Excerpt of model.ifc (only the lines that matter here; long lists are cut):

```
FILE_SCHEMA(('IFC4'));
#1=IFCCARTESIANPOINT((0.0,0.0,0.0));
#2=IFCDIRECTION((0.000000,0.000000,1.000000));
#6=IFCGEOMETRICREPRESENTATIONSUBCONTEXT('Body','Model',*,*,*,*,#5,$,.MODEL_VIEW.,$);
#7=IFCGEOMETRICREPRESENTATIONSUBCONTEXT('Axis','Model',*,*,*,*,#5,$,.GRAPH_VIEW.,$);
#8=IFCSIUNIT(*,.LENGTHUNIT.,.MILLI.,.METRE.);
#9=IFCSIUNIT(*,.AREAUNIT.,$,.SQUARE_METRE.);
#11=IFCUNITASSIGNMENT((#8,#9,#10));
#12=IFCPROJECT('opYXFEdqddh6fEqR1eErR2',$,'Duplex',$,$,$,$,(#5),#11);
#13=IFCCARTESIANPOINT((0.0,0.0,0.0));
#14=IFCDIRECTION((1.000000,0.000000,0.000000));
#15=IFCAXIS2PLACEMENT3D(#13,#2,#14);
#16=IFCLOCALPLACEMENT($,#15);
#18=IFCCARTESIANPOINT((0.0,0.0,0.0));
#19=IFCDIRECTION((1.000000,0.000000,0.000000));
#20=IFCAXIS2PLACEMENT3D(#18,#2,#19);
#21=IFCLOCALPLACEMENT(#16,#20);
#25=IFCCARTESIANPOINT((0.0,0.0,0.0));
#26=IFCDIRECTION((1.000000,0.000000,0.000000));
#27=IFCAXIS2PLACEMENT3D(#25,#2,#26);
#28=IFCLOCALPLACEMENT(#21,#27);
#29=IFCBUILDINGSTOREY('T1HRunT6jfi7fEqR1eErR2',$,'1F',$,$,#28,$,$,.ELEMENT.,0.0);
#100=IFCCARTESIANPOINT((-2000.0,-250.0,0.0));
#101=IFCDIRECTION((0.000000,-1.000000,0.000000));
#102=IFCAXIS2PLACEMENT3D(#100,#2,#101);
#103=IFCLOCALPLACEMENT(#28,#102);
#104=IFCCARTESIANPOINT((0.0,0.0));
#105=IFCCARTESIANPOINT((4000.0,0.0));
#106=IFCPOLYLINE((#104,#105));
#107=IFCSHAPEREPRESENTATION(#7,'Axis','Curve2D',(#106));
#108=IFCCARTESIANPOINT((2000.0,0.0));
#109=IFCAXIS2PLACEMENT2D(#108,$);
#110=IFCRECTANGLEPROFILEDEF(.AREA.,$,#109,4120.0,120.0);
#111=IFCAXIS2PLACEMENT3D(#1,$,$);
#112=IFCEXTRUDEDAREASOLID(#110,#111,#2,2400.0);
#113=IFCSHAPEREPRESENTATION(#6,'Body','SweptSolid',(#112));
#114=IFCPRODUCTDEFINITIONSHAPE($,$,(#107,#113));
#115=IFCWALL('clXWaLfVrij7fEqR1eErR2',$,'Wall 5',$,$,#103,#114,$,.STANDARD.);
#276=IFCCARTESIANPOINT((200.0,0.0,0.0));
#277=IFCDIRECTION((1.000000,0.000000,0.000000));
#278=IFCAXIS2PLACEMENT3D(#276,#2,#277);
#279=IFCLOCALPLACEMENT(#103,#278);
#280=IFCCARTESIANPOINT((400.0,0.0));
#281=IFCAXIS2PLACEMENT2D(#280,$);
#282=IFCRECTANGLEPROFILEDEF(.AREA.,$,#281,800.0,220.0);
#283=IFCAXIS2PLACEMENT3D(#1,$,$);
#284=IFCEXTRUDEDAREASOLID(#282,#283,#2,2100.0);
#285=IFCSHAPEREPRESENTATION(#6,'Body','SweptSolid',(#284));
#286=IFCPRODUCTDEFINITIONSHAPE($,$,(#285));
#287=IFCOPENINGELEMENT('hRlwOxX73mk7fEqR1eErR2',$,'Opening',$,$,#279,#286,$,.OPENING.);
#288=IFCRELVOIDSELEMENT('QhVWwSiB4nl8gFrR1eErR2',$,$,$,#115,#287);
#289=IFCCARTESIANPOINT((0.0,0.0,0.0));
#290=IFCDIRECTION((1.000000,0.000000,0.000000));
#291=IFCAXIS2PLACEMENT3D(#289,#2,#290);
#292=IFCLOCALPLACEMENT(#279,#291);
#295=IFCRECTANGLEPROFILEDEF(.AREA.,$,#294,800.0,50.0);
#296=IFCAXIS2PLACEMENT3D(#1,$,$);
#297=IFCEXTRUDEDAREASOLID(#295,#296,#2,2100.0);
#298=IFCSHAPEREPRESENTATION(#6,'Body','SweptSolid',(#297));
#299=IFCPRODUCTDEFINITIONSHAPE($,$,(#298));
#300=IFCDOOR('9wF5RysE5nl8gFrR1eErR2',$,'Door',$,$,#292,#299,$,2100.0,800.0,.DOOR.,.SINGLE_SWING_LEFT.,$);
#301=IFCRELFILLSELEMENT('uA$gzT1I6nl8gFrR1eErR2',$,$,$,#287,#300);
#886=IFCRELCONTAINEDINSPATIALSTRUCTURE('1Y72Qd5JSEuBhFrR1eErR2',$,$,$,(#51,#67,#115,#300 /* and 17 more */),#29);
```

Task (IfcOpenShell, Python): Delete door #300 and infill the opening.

```python
import ifcopenshell
import ifcopenshell.api.feature
import ifcopenshell.api.root
import ifcopenshell.geom
import ifcopenshell.util.shape

model = ifcopenshell.open("model.ifc")
settings = ifcopenshell.geom.settings()


def volume(element):
    """Net volume in cubic metres, openings subtracted."""
    shape = ifcopenshell.geom.create_shape(settings, element)
    return ifcopenshell.util.shape.get_volume(shape.geometry)


door = model.by_guid("9wF5RysE5nl8gFrR1eErR2")
opening = door.FillsVoids[0].RelatingOpeningElement
wall = opening.VoidsElements[0].RelatingBuildingElement
before = volume(wall)

ifcopenshell.api.root.remove_product(model, product=door)
ifcopenshell.api.feature.remove_feature(model, feature=opening)

after = volume(wall)

print(f"wall volume {before:.3f} -> {after:.3f} m3")

model.write("model_edited.ifc")
```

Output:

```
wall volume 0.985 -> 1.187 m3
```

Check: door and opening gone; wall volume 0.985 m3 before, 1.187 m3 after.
